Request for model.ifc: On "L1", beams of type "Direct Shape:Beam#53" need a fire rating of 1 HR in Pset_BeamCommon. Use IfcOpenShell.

First a look at what the model holds.

```python
import ifcopenshell
import ifcopenshell.util.element

model = ifcopenshell.open("model.ifc")
print(model.schema)
storey = next(s for s in model.by_type("IfcBuildingStorey") if s.Name == "L1")
beams = [e for e in ifcopenshell.util.element.get_decomposition(storey) if e.is_a("IfcBeam")]
seen = {}
for e in beams:
    element_type = ifcopenshell.util.element.get_type(e)
    key = (element_type.Name if element_type != e and element_type else None, ifcopenshell.util.element.get_pset(e, "Pset_BeamCommon", "FireRating"))
    seen[key] = seen.get(key, 0) + 1
for (name, value), count in sorted(seen.items(), key=str):
    print(count, "x", name, "|", value)
```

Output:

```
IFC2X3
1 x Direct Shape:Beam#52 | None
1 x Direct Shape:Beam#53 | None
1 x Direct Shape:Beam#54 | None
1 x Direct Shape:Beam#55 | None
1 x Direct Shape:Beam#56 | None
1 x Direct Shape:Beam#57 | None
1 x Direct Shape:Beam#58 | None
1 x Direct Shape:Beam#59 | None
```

```python
import ifcopenshell
import ifcopenshell.api.pset
import ifcopenshell.util.element

model = ifcopenshell.open("model.ifc")

storey = next(s for s in model.by_type("IfcBuildingStorey") if s.Name == "L1")
beams = [e for e in ifcopenshell.util.element.get_decomposition(storey) if e.is_a("IfcBeam")]

count = 0
for e in beams:
    element_type = ifcopenshell.util.element.get_type(e)
    if element_type in (None, e) or element_type.Name != "Direct Shape:Beam#53":
        continue
    # add_pset returns the element's existing set when there is one.
    pset = ifcopenshell.api.pset.add_pset(model, product=e, name="Pset_BeamCommon")
    ifcopenshell.api.pset.edit_pset(model, pset=pset, properties={"FireRating": "1 HR"})
    count += 1

print(count, "beams updated")

model.write("model_edited.ifc")
```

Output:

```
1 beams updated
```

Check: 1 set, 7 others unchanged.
